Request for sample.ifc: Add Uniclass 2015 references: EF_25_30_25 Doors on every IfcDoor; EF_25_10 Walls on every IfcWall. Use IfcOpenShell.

First a look at what the model holds.

```python
import ifcopenshell

model = ifcopenshell.open("sample.ifc")
print(model.schema)
print("classifications:", [c.Name for c in model.by_type("IfcClassification")])
for ifc_class in ("IfcDoor", "IfcRoof", "IfcStair", "IfcWall", "IfcWindow"):
    print(ifc_class, len(model.by_type(ifc_class)))
```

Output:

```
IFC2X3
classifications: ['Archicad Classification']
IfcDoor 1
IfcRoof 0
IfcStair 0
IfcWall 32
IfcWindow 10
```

```python
import ifcopenshell
import ifcopenshell.api.classification

model = ifcopenshell.open("sample.ifc")

# IFC2X3 requires Source and Edition and has no link from the project to the system.
system = model.create_entity("IfcClassification", Source="NBS", Edition="2015", Name="Uniclass 2015")

codes = {
    "IfcDoor": ("EF_25_30_25", "Doors"),
    "IfcWall": ("EF_25_10", "Walls"),
}
for ifc_class, (code, name) in codes.items():
    products = model.by_type(ifc_class)
    ifcopenshell.api.classification.add_reference(
        model, products=products, classification=system, identification=code, name=name
    )
    print(code, len(products))

model.write("sample_v2.ifc")
```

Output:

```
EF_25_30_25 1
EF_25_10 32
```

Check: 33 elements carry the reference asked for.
